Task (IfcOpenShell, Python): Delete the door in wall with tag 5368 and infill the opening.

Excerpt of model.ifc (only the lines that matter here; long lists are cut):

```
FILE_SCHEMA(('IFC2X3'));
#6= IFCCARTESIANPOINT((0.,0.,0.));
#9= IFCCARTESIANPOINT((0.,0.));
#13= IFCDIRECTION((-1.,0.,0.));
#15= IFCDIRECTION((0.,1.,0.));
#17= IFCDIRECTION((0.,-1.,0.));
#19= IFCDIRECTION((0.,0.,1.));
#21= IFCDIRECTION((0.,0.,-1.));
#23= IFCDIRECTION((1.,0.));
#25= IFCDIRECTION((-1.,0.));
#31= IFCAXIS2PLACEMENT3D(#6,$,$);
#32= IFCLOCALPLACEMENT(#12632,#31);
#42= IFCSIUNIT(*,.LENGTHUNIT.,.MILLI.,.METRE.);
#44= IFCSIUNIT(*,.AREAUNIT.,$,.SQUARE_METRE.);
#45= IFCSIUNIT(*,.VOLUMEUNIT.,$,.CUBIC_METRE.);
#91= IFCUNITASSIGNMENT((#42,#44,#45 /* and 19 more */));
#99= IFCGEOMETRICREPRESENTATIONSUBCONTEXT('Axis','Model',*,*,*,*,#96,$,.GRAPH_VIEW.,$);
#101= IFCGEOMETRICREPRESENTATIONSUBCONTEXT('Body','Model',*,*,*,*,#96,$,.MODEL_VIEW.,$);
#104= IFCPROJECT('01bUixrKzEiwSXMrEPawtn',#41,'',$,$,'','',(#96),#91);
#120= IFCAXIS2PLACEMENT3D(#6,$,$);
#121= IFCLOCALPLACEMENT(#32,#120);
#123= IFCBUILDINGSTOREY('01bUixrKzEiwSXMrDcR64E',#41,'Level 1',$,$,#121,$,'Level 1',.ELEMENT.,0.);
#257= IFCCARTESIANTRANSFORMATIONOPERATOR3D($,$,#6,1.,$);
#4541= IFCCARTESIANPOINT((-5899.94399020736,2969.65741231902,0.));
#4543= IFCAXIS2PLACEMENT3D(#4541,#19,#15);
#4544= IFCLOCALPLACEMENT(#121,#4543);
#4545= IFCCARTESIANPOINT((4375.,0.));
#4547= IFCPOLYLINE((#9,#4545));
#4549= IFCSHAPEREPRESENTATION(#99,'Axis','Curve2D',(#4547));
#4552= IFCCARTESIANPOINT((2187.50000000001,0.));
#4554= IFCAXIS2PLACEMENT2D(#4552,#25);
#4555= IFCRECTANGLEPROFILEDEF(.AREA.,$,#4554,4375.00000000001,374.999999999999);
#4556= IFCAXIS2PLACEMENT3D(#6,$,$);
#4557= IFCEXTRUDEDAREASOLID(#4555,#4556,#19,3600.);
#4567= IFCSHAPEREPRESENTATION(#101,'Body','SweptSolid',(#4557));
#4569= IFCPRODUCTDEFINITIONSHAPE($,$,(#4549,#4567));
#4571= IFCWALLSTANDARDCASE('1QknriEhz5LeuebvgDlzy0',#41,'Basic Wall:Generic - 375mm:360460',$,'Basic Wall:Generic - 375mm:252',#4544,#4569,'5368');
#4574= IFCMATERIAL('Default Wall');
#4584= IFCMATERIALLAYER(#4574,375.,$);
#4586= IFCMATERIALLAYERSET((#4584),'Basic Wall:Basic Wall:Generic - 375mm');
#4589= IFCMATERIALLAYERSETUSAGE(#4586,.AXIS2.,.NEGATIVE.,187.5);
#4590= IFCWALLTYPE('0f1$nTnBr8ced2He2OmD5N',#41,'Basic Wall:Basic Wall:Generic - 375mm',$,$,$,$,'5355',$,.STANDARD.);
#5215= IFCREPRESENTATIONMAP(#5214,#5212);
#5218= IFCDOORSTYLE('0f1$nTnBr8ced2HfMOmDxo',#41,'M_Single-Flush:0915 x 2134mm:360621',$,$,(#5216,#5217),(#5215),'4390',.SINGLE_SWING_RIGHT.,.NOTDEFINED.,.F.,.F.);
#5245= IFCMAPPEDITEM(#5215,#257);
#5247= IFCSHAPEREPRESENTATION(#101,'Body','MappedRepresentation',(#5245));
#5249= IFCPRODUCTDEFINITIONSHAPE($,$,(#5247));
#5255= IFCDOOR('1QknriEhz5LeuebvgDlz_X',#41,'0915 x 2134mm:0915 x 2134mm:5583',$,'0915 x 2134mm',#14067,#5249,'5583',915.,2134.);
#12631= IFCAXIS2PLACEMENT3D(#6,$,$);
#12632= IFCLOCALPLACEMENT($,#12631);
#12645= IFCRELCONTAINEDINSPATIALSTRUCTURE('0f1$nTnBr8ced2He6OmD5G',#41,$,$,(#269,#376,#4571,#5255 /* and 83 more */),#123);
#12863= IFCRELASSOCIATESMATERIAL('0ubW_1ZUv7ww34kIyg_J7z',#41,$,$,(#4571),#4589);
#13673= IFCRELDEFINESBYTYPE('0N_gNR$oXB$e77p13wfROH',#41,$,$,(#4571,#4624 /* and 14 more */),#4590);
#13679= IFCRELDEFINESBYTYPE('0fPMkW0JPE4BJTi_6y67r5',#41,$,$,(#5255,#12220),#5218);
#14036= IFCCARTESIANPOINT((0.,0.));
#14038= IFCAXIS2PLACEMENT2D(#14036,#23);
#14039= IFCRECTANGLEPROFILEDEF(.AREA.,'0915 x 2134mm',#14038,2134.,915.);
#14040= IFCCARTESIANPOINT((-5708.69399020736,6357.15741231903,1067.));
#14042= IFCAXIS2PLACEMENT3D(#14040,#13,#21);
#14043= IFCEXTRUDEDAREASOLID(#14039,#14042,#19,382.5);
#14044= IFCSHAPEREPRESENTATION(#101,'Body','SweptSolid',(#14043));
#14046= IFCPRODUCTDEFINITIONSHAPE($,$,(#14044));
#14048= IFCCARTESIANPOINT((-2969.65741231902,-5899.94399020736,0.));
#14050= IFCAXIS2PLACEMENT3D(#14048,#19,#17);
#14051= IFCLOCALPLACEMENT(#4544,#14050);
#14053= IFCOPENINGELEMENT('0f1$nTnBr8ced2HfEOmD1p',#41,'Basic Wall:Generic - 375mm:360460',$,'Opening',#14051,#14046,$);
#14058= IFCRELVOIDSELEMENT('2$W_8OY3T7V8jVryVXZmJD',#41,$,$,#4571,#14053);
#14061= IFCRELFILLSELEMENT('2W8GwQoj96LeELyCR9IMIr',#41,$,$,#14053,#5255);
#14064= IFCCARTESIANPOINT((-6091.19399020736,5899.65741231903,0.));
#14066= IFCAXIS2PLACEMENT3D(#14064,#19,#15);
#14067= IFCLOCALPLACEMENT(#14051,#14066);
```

```python
import ifcopenshell
import ifcopenshell.api.feature
import ifcopenshell.api.root
import ifcopenshell.geom
import ifcopenshell.util.shape

model = ifcopenshell.open("model.ifc")
settings = ifcopenshell.geom.settings()


def volume(element):
    """Net volume in cubic metres, openings subtracted."""
    shape = ifcopenshell.geom.create_shape(settings, element)
    return ifcopenshell.util.shape.get_volume(shape.geometry)


door = model.by_guid("1QknriEhz5LeuebvgDlz_X")
opening = door.FillsVoids[0].RelatingOpeningElement
wall = opening.VoidsElements[0].RelatingBuildingElement
before = volume(wall)

ifcopenshell.api.root.remove_product(model, product=door)
ifcopenshell.api.feature.remove_feature(model, feature=opening)

after = volume(wall)

print(f"wall volume {before:.3f} -> {after:.3f} m3")

model.write("model-out.ifc")
```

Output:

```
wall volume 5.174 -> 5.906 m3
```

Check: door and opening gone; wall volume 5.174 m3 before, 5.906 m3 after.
